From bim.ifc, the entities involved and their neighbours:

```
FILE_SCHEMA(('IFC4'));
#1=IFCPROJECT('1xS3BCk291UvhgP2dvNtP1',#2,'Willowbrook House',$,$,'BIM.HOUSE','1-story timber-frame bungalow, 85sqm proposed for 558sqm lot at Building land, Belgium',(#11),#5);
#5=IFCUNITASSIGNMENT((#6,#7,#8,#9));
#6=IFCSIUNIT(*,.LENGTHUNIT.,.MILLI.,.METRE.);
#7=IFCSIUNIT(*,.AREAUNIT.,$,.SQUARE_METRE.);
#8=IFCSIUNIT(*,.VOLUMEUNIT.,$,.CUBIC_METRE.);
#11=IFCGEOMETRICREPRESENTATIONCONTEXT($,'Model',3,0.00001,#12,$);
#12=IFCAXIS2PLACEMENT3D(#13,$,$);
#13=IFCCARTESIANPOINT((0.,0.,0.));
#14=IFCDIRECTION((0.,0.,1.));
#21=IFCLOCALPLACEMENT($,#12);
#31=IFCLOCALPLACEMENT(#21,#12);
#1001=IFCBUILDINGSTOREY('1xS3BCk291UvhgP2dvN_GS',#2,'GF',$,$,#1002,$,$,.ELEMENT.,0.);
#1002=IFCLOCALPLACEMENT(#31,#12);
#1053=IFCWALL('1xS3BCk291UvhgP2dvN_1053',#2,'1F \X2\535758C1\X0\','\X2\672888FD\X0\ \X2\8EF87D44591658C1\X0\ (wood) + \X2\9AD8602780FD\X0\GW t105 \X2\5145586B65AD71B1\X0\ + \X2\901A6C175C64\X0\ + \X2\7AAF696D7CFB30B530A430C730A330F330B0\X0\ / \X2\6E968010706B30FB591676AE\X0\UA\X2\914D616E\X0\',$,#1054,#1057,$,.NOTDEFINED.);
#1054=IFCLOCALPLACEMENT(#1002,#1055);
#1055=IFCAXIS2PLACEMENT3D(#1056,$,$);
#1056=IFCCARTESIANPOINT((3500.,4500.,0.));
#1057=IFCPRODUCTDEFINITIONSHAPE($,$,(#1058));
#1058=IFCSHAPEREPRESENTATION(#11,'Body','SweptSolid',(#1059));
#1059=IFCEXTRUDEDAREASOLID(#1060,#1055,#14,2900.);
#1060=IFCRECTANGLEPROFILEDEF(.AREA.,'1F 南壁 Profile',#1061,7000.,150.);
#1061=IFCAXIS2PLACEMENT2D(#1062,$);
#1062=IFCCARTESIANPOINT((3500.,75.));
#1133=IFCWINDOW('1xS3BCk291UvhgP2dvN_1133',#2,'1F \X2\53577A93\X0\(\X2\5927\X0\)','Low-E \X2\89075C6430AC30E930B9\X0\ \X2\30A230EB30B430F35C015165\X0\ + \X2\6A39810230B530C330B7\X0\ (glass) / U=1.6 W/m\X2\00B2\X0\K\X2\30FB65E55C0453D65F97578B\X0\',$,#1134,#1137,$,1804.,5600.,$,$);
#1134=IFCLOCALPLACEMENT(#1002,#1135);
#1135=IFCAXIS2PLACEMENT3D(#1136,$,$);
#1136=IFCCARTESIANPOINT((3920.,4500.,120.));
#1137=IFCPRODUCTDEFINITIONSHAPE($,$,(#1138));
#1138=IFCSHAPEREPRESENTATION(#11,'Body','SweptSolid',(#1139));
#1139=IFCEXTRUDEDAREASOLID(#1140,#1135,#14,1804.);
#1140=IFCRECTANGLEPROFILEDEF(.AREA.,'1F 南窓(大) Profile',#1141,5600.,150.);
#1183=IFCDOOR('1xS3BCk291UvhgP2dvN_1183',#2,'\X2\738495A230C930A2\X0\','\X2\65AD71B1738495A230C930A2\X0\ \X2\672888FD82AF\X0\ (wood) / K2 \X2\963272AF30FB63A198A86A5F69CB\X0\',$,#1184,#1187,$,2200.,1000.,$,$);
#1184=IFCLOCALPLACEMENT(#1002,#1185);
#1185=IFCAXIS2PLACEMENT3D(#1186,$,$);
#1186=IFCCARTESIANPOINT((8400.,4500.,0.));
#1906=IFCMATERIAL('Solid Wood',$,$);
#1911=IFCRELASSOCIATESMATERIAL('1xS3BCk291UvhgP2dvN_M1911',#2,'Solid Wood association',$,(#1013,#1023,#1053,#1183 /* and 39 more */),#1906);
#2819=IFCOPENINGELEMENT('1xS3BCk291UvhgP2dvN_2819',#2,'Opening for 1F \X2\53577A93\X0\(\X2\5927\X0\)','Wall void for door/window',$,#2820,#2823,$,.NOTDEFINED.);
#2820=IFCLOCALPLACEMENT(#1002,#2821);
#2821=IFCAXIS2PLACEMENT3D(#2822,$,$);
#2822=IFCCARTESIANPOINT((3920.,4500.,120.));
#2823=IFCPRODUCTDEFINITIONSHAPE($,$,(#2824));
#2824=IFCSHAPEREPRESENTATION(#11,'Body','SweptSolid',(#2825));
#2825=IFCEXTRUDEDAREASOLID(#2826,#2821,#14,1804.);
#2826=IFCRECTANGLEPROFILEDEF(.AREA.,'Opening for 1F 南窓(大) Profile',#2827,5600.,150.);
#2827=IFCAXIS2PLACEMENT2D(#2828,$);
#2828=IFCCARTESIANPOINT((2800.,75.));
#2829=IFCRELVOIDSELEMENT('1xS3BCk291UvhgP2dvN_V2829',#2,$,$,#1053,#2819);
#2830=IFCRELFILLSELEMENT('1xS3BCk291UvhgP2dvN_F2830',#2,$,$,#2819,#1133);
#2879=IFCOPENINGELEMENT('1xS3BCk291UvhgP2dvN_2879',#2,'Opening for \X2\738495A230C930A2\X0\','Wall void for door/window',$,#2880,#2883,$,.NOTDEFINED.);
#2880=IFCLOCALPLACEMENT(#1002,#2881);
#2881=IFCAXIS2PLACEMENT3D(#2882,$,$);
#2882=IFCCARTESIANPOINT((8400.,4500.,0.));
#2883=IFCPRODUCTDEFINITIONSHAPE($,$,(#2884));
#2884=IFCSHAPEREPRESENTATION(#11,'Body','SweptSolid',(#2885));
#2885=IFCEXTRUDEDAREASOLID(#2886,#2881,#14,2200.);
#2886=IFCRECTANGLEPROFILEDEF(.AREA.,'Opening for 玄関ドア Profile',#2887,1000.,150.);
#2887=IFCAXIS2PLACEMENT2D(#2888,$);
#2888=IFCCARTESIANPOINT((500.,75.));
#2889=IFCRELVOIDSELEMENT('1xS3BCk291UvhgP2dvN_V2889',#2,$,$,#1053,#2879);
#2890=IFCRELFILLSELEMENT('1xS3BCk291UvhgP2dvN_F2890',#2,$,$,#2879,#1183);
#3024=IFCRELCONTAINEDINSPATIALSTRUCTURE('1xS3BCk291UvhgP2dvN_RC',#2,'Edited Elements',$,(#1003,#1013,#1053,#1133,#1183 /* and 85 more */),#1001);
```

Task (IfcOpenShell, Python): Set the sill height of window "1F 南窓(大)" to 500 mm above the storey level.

```python
import numpy as np
import ifcopenshell
import ifcopenshell.api.geometry
import ifcopenshell.geom
import ifcopenshell.util.element
import ifcopenshell.util.placement
import ifcopenshell.util.shape
import ifcopenshell.util.unit

model = ifcopenshell.open("bim.ifc")
unit_scale = ifcopenshell.util.unit.calculate_unit_scale(model)

window = model.by_guid("1xS3BCk291UvhgP2dvN_1133")
opening = window.FillsVoids[0].RelatingOpeningElement
storey = ifcopenshell.util.element.get_container(window, ifc_class="IfcBuildingStorey")
level = ifcopenshell.util.placement.get_local_placement(storey.ObjectPlacement)[2, 3]

# The opening's origin need not be at the sill, so measure its lowest point.
shape = ifcopenshell.geom.create_shape(ifcopenshell.geom.settings(), opening)
bottom = ifcopenshell.util.shape.get_shape_bottom_elevation(shape, shape.geometry) / unit_scale
dz = level + 0.5 / unit_scale - bottom

shift = np.array([0.0, 0.0, dz])
# The window is not placed relative to its opening, so move both.
for product in (opening, window):
    matrix = ifcopenshell.util.placement.get_local_placement(product.ObjectPlacement)
    matrix[:3, 3] += shift
    ifcopenshell.api.geometry.edit_object_placement(model, product=product, matrix=matrix, is_si=False)

print(f"moved by {dz * unit_scale:+.3f} m")

model.write("bim_updated.ifc")
```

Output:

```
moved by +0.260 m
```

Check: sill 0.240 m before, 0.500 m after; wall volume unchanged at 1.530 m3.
